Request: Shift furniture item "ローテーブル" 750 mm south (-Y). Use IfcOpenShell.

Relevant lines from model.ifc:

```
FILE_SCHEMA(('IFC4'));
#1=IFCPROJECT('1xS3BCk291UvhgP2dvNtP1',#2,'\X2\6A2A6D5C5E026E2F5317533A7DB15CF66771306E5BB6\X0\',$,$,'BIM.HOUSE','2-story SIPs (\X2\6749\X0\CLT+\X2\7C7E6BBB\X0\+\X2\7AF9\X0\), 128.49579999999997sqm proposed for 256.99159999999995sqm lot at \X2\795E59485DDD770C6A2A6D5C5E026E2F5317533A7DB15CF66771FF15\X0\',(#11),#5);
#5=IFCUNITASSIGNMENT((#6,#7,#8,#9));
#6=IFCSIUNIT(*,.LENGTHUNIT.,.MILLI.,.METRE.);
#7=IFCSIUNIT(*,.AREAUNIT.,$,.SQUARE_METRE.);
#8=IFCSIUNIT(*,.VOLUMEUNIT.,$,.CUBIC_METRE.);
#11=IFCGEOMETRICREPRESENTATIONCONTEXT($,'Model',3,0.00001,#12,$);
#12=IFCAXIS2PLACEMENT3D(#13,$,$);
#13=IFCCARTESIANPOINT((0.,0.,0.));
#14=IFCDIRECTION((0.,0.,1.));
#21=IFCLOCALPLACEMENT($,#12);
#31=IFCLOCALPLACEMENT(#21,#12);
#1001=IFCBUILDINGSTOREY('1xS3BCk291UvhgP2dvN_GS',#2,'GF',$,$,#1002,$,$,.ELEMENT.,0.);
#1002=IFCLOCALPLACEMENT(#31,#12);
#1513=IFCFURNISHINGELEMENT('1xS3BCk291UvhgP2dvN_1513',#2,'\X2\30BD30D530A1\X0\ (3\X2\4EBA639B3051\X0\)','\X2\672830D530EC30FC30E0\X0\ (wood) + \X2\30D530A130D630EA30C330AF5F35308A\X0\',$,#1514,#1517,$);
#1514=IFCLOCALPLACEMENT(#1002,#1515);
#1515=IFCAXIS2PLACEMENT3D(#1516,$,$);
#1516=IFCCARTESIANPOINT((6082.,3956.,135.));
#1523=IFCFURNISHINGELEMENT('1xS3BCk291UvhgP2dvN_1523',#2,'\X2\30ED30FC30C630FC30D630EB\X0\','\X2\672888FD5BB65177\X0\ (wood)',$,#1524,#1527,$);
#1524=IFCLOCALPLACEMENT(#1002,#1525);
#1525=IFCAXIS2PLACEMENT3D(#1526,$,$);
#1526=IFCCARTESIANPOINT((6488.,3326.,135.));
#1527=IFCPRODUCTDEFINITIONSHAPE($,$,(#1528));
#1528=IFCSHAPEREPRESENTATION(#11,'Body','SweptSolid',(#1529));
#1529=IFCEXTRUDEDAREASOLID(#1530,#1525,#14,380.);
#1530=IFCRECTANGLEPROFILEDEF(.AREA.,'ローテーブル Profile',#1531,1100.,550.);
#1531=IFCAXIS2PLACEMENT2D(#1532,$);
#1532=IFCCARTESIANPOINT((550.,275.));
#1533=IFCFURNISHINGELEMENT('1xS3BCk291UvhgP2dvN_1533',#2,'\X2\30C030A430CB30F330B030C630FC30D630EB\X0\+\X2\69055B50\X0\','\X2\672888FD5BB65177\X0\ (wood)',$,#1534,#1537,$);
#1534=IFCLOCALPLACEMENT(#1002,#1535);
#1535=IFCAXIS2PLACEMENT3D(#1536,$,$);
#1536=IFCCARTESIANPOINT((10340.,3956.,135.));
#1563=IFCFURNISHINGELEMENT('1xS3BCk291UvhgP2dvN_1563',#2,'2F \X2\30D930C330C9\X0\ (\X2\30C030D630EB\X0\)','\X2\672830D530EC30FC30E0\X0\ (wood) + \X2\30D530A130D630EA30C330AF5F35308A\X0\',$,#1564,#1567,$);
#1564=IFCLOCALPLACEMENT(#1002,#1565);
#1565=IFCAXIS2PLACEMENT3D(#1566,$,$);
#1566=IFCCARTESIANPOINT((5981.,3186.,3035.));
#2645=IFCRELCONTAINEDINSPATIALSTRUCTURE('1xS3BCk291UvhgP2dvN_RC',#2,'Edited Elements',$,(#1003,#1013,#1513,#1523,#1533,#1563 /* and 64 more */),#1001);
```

```python
import ifcopenshell
import ifcopenshell.api.geometry
import ifcopenshell.util.placement

model = ifcopenshell.open("model.ifc")

item = model.by_guid("1xS3BCk291UvhgP2dvN_1523")
matrix = ifcopenshell.util.placement.get_local_placement(item.ObjectPlacement)
matrix[1, 3] -= 750.0
ifcopenshell.api.geometry.edit_object_placement(model, product=item, matrix=matrix, is_si=False)

print(ifcopenshell.util.placement.get_local_placement(item.ObjectPlacement).round(3) + 0.0)

model.write("model_v2.ifc")
```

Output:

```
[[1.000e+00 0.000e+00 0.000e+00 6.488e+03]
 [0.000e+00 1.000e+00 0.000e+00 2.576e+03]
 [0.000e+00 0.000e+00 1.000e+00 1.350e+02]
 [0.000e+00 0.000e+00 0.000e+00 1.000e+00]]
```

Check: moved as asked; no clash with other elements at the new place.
